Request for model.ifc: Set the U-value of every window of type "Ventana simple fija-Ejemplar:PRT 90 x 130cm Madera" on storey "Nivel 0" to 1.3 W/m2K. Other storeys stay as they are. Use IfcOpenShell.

First a look at what the model holds.

```python
import ifcopenshell
import ifcopenshell.util.element

model = ifcopenshell.open("model.ifc")
print(model.schema)
storey = next(s for s in model.by_type("IfcBuildingStorey") if s.Name == "Nivel 0")
windows = [e for e in ifcopenshell.util.element.get_decomposition(storey) if e.is_a("IfcWindow")]
seen = {}
for e in windows:
    element_type = ifcopenshell.util.element.get_type(e)
    key = (element_type.Name if element_type != e and element_type else None, ifcopenshell.util.element.get_pset(e, "Pset_WindowCommon", "ThermalTransmittance"))
    seen[key] = seen.get(key, 0) + 1
for (name, value), count in sorted(seen.items(), key=str):
    print(count, "x", name, "|", value)
```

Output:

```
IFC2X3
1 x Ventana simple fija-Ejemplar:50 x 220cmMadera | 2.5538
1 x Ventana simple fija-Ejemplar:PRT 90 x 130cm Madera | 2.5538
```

```python
import ifcopenshell
import ifcopenshell.api.pset
import ifcopenshell.util.element

model = ifcopenshell.open("model.ifc")

storey = next(s for s in model.by_type("IfcBuildingStorey") if s.Name == "Nivel 0")
windows = [e for e in ifcopenshell.util.element.get_decomposition(storey) if e.is_a("IfcWindow")]

count = 0
for e in windows:
    element_type = ifcopenshell.util.element.get_type(e)
    if element_type in (None, e) or element_type.Name != "Ventana simple fija-Ejemplar:PRT 90 x 130cm Madera":
        continue
    # add_pset returns the element's existing set when there is one.
    pset = ifcopenshell.api.pset.add_pset(model, product=e, name="Pset_WindowCommon")
    ifcopenshell.api.pset.edit_pset(model, pset=pset, properties={"ThermalTransmittance": 1.3})
    count += 1

print(count, "windows updated")

model.write("model-out.ifc")
```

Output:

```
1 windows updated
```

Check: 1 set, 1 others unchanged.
